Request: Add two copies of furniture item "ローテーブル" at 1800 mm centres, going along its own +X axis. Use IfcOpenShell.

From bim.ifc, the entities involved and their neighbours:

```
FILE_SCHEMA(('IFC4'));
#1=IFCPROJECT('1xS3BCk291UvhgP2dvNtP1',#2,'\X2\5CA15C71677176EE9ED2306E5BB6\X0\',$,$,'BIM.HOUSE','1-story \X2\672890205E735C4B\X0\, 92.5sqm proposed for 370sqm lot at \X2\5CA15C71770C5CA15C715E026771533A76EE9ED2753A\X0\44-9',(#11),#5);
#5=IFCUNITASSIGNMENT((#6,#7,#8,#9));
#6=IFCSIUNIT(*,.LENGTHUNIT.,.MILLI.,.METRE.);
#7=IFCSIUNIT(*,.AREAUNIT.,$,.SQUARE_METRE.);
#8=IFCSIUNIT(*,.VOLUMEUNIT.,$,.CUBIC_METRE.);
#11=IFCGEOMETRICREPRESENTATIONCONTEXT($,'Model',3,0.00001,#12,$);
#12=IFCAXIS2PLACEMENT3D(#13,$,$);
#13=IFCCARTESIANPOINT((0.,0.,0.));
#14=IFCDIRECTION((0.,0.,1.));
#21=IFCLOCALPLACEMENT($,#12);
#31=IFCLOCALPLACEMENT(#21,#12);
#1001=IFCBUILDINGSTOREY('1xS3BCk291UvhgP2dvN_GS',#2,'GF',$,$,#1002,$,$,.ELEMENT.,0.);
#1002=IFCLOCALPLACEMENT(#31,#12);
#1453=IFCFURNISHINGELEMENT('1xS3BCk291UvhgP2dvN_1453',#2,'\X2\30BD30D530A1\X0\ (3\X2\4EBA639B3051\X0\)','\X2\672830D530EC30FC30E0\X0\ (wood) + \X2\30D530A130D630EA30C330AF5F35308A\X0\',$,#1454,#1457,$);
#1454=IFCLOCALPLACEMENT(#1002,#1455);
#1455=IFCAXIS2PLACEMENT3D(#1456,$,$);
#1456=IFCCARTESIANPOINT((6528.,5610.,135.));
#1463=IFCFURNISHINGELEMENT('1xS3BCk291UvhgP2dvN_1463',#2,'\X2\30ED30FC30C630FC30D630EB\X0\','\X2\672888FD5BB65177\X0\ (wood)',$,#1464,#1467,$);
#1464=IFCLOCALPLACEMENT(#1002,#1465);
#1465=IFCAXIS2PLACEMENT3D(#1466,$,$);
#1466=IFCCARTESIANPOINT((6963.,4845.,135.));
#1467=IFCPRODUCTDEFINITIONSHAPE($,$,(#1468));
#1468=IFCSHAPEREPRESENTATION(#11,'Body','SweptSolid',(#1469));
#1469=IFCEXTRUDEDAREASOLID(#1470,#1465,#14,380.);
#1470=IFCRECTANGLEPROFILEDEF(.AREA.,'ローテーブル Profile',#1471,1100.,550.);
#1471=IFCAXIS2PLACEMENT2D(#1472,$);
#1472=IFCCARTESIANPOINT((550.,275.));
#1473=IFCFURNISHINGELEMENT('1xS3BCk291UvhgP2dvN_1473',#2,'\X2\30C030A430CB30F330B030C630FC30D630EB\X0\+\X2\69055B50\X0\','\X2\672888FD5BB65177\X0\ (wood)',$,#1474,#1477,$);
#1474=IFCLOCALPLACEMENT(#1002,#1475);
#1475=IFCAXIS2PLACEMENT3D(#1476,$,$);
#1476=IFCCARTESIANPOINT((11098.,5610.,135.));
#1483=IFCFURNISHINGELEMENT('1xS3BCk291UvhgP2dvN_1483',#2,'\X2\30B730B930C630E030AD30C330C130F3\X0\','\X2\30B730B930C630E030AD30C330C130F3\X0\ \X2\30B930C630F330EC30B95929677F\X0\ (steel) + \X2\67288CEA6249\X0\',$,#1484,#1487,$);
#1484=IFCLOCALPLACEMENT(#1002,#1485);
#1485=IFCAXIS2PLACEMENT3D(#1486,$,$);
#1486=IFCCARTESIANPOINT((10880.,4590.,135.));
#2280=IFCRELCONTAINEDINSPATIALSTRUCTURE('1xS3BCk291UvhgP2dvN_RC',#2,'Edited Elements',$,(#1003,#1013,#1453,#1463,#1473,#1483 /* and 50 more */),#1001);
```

```python
import ifcopenshell
import ifcopenshell.api.geometry
import ifcopenshell.api.root
import ifcopenshell.util.element
import ifcopenshell.util.placement

model = ifcopenshell.open("bim.ifc")


def reuse_history(source, copy):
    """copy_class also copies each property set's owner history, people and application; keep the originals."""
    for rel in copy.IsDefinedBy:
        if rel.is_a("IfcRelDefinesByProperties") and (history := rel.RelatingPropertyDefinition.OwnerHistory):
            rel.RelatingPropertyDefinition.OwnerHistory = source.OwnerHistory
            ifcopenshell.util.element.remove_deep2(model, history)


source = model.by_guid("1xS3BCk291UvhgP2dvN_1463")
base = ifcopenshell.util.placement.get_local_placement(source.ObjectPlacement)
step = base[:3, 0] * 1800.0

for i in range(1, 3):
    copy = ifcopenshell.api.root.copy_class(model, product=source)
    copy.Representation = ifcopenshell.util.element.copy_deep(
        model, source.Representation, exclude=["IfcGeometricRepresentationContext", "IfcRepresentationMap"]
    )
    reuse_history(source, copy)
    matrix = base.copy()
    matrix[:3, 3] += i * step
    print("added at", matrix[:3, 3].round(3) + 0.0)
    ifcopenshell.api.geometry.edit_object_placement(model, product=copy, matrix=matrix, is_si=False)

model.write("bim_v2.ifc")
```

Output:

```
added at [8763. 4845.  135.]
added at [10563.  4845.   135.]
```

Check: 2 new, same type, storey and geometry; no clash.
